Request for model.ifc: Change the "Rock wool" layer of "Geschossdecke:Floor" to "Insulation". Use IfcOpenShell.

First a look at what the model holds.

```python
import ifcopenshell
import ifcopenshell.util.element

model = ifcopenshell.open("model.ifc")
print(model.schema)
for layer_set in model.by_type("IfcMaterialLayerSet"):
    if layer_set.LayerSetName == "Geschossdecke:Floor":
        for layer in layer_set.MaterialLayers:
            print(layer.id(), layer.Material and layer.Material.Name, layer.LayerThickness, sep=" | ")
        print(len(ifcopenshell.util.element.get_elements_by_material(model, layer_set)), "elements and types use it")
print(sorted(m.Name for m in model.by_type("IfcMaterial") if m.Name)[:60])
```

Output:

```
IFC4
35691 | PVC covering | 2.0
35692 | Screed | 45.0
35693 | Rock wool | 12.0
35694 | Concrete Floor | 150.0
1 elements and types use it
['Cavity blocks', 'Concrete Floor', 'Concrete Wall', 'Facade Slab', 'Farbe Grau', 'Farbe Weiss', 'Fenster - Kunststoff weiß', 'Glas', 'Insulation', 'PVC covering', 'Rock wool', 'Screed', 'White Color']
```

```python
import ifcopenshell
import ifcopenshell.api.material

model = ifcopenshell.open("model.ifc")

layer_set = next(s for s in model.by_type("IfcMaterialLayerSet") if s.LayerSetName == "Geschossdecke:Floor")
layer = next(l for l in layer_set.MaterialLayers if l.Material and l.Material.Name == "Rock wool")
material = next(m for m in model.by_type("IfcMaterial") if m.Name == "Insulation")

# Point this one layer at the other material; renaming the old one would change it everywhere.
ifcopenshell.api.material.edit_layer(model, layer=layer, attributes={}, material=material)

print([l.Material.Name if l.Material else None for l in layer_set.MaterialLayers])

model.write("model_rev.ifc")
```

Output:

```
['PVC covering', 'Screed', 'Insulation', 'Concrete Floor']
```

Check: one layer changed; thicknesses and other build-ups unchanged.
